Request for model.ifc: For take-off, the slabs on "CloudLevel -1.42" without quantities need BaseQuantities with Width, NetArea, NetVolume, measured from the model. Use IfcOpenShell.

First a look at what the model holds.

```python
import ifcopenshell
import ifcopenshell.util.element
import ifcopenshell.util.unit

model = ifcopenshell.open("model.ifc")
print(model.schema)
for unit_type in ("LENGTHUNIT", "AREAUNIT", "VOLUMEUNIT"):
    print(unit_type, ifcopenshell.util.unit.calculate_unit_scale(model, unit_type))
storey = next(s for s in model.by_type("IfcBuildingStorey") if s.Name == "CloudLevel -1.42")
slabs = [e for e in ifcopenshell.util.element.get_decomposition(storey) if e.is_a("IfcSlab")]
for e in sorted(slabs, key=lambda e: e.id()):
    print(e.id(), e.is_a(), e.Name, list(ifcopenshell.util.element.get_psets(e, qtos_only=True)), sep=" | ")
```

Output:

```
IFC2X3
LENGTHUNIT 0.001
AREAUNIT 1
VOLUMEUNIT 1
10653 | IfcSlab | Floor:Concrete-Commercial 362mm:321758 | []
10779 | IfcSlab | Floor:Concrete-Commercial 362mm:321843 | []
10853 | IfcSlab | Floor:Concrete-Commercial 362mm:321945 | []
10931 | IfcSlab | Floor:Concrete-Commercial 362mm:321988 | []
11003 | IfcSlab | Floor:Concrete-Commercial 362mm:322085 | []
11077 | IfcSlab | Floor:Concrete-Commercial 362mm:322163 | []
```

```python
import ifcopenshell
import ifcopenshell.api.pset
import ifcopenshell.geom
import ifcopenshell.util.element
import ifcopenshell.util.shape
import ifcopenshell.util.unit

model = ifcopenshell.open("model.ifc")
unit_scale = ifcopenshell.util.unit.calculate_unit_scale(model)
area_scale = ifcopenshell.util.unit.calculate_unit_scale(model, "AREAUNIT")
volume_scale = ifcopenshell.util.unit.calculate_unit_scale(model, "VOLUMEUNIT")
settings = ifcopenshell.geom.settings()

storey = next(s for s in model.by_type("IfcBuildingStorey") if s.Name == "CloudLevel -1.42")
slabs = [e for e in ifcopenshell.util.element.get_decomposition(storey) if e.is_a("IfcSlab")]

for e in sorted(slabs, key=lambda e: e.id()):
    if ifcopenshell.util.element.get_psets(e, qtos_only=True, should_inherit=False):
        continue
    # Geometry comes back in metres, in the element's own axes.
    shape = ifcopenshell.geom.create_shape(settings, e)
    values = {
        "Width": ifcopenshell.util.shape.get_z(shape.geometry) / unit_scale,
        "NetArea": ifcopenshell.util.shape.get_footprint_area(shape.geometry) / area_scale,
        "NetVolume": ifcopenshell.util.shape.get_volume(shape.geometry) / volume_scale,
    }
    qto = ifcopenshell.api.pset.add_qto(model, product=e, name="BaseQuantities")
    ifcopenshell.api.pset.edit_qto(model, qto=qto, properties=values)
    print(e.id(), {k: round(v, 3) for k, v in values.items()})

model.write("model-out.ifc")
```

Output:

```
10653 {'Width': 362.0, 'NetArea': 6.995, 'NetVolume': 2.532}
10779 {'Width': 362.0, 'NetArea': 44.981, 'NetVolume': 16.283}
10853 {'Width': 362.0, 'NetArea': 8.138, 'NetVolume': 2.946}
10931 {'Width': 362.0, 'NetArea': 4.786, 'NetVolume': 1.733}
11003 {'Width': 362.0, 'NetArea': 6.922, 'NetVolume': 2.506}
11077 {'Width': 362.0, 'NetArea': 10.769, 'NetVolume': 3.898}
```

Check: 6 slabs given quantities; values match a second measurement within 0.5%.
